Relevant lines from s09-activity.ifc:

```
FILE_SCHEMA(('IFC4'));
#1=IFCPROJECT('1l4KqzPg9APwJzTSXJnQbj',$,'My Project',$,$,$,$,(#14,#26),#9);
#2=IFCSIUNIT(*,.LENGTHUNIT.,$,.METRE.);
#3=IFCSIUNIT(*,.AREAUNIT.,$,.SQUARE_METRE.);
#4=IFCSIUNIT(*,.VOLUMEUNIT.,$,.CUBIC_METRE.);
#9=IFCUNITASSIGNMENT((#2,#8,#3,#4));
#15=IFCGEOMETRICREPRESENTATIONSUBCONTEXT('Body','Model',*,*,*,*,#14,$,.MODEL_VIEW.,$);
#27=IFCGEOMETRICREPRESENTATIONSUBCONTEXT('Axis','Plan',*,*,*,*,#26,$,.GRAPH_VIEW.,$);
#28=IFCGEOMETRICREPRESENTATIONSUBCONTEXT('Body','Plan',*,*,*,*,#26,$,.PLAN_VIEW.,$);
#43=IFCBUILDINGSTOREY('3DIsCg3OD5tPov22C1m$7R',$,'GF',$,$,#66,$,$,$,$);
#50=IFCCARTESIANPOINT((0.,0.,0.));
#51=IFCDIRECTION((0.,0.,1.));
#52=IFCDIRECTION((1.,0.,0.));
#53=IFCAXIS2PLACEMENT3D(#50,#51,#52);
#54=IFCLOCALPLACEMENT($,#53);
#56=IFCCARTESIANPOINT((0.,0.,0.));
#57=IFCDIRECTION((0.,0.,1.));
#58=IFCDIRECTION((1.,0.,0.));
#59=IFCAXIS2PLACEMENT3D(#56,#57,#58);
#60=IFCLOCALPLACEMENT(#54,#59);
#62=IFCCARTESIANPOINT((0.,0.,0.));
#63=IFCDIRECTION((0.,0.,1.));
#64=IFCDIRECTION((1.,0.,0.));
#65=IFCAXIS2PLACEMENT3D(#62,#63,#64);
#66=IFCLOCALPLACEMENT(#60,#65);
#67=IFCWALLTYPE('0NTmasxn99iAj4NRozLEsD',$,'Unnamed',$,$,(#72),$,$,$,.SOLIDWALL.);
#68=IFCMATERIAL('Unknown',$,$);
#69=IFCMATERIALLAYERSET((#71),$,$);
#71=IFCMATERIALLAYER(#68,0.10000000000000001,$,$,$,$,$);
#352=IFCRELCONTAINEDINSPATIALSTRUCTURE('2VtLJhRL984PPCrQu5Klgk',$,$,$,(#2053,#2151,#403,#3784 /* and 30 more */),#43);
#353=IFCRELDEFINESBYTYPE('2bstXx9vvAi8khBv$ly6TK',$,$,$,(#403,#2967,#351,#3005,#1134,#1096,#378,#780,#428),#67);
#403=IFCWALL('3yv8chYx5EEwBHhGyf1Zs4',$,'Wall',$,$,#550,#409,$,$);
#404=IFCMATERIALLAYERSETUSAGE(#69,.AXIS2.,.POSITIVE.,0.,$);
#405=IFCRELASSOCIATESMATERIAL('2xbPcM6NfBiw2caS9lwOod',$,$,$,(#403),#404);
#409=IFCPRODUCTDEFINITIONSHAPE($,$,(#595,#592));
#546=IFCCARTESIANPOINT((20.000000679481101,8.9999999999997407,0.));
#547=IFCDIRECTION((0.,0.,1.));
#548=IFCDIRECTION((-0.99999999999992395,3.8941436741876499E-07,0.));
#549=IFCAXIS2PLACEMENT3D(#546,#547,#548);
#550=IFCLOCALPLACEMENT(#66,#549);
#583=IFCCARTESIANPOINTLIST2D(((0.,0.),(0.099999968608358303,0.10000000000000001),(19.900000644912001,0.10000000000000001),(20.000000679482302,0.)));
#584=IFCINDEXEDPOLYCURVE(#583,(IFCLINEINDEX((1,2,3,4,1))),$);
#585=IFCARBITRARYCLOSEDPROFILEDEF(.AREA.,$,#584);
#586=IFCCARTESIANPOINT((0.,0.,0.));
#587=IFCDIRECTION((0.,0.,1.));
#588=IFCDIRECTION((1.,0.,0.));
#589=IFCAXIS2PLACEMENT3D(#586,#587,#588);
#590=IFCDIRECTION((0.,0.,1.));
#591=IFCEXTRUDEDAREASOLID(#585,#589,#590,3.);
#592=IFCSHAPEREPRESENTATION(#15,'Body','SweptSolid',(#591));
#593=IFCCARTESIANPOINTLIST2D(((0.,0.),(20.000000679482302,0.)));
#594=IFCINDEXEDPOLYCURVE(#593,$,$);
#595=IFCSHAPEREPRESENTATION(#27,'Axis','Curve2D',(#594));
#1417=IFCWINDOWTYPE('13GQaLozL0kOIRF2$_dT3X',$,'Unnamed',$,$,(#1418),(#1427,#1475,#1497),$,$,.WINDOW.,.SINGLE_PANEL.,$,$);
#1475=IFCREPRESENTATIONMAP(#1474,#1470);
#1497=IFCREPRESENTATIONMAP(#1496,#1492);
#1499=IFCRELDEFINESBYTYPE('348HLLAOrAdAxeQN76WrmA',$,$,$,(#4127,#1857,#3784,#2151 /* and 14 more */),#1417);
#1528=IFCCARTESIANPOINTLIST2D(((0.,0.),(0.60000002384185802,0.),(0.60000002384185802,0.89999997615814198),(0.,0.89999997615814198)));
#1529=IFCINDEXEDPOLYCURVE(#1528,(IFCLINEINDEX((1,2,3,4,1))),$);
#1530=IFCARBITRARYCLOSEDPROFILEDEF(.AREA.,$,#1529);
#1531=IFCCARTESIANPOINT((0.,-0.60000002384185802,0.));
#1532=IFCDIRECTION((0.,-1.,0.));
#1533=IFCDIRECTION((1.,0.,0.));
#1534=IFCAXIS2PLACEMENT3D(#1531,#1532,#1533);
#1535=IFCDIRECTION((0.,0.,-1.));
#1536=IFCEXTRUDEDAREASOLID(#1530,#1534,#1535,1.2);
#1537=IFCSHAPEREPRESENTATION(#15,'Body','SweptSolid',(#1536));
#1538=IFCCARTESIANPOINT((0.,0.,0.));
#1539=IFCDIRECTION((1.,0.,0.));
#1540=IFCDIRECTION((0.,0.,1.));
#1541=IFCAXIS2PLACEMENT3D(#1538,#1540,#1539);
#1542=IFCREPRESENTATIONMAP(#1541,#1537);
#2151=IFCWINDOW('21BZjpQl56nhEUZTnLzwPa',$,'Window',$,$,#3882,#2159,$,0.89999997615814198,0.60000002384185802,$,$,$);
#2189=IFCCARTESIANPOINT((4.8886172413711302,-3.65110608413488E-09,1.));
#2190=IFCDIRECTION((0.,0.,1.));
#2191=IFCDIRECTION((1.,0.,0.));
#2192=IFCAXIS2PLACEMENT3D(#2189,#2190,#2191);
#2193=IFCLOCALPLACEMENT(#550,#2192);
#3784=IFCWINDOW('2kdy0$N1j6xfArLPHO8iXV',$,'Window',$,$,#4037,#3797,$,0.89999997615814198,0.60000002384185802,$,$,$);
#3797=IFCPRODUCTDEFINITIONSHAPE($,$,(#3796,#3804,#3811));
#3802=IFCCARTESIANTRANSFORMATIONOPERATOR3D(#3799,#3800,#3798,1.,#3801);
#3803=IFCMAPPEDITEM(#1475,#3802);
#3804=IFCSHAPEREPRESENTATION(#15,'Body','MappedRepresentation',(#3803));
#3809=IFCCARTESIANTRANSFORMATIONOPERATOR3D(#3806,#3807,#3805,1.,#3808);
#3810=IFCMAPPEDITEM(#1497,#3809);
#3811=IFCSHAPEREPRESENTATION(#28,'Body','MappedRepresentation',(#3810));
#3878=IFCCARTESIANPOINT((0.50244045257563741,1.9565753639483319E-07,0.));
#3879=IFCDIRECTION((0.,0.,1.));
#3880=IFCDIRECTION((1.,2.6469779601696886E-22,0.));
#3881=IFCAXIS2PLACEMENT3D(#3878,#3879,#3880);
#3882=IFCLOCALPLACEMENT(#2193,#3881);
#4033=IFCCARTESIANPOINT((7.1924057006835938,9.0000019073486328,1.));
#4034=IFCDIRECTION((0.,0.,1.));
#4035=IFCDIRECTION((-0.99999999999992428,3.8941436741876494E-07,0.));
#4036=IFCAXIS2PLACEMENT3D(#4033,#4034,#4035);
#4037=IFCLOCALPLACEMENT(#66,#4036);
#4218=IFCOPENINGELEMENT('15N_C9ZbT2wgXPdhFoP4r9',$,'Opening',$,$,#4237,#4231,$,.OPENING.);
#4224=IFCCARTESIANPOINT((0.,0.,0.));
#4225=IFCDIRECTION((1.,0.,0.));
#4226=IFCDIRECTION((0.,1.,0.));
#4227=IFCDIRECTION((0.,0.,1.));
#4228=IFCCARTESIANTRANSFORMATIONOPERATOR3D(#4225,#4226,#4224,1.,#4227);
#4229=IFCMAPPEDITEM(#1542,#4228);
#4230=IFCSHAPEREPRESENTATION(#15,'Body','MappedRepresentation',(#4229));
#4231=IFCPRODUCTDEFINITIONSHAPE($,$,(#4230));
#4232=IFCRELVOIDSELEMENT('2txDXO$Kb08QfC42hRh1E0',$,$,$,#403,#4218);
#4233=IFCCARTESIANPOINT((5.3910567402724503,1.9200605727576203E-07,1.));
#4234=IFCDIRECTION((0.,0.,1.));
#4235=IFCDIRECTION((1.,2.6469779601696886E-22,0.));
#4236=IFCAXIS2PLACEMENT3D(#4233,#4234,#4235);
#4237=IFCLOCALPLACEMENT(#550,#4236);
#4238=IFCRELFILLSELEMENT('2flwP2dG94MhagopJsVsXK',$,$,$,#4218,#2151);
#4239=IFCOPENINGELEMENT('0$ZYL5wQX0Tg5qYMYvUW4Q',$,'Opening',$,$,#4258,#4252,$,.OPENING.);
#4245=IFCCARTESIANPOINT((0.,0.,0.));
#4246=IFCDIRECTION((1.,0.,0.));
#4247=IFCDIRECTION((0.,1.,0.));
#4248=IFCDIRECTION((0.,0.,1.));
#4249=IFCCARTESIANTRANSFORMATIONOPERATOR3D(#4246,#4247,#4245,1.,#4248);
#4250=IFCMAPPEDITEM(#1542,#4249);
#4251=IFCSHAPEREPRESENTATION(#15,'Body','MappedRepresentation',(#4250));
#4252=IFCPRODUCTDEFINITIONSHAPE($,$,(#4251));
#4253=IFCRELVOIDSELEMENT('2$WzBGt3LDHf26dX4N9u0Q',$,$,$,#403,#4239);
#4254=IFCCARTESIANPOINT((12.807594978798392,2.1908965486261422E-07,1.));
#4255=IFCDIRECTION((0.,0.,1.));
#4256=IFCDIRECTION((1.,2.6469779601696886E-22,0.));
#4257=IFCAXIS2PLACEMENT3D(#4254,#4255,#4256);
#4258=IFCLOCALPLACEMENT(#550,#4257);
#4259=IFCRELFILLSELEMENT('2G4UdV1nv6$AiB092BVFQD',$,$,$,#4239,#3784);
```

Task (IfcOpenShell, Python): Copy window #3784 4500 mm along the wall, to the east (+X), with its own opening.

```python
import ifcopenshell
import ifcopenshell.api.feature
import ifcopenshell.api.geometry
import ifcopenshell.api.root
import ifcopenshell.geom
import ifcopenshell.util.element
import ifcopenshell.util.placement
import ifcopenshell.util.shape

model = ifcopenshell.open("s09-activity.ifc")
settings = ifcopenshell.geom.settings()


def volume(element):
    """Net volume in cubic metres, openings subtracted."""
    shape = ifcopenshell.geom.create_shape(settings, element)
    return ifcopenshell.util.shape.get_volume(shape.geometry)


window = model.by_guid("2kdy0$N1j6xfArLPHO8iXV")
opening = window.FillsVoids[0].RelatingOpeningElement
wall = opening.VoidsElements[0].RelatingBuildingElement
before = volume(wall)
shift = ifcopenshell.util.placement.get_local_placement(wall.ObjectPlacement)[:3, 0] * -4.5

# copy_class copies the void relationship, type, container and properties, but no geometry.
new_opening = ifcopenshell.api.root.copy_class(model, product=opening)
new_opening.Representation = ifcopenshell.util.element.copy_deep(
    model, opening.Representation, exclude=["IfcGeometricRepresentationContext", "IfcRepresentationMap"]
)
new_window = ifcopenshell.api.root.copy_class(model, product=window)
new_window.Representation = ifcopenshell.util.element.copy_deep(
    model, window.Representation, exclude=["IfcGeometricRepresentationContext", "IfcRepresentationMap"]
)
ifcopenshell.api.feature.add_filling(model, opening=new_opening, element=new_window)

for old, new in ((opening, new_opening), (window, new_window)):
    matrix = ifcopenshell.util.placement.get_local_placement(old.ObjectPlacement)
    matrix[:3, 3] += shift
    ifcopenshell.api.geometry.edit_object_placement(model, product=new, matrix=matrix, is_si=False)

after = volume(wall)

print(f"wall volume {before:.3f} -> {after:.3f} m3")

model.write("s09-activity-out.ifc")
```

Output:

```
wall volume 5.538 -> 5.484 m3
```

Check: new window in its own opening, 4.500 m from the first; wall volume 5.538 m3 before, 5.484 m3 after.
